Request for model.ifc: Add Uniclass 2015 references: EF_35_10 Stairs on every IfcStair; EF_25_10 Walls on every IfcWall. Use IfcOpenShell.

First a look at what the model holds.

```python
import ifcopenshell

model = ifcopenshell.open("model.ifc")
print(model.schema)
print("classifications:", [c.Name for c in model.by_type("IfcClassification")])
for ifc_class in ("IfcDoor", "IfcRoof", "IfcStair", "IfcWall", "IfcWindow"):
    print(ifc_class, len(model.by_type(ifc_class)))
```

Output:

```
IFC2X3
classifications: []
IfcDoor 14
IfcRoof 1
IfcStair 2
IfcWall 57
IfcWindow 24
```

```python
import ifcopenshell
import ifcopenshell.api.classification

model = ifcopenshell.open("model.ifc")

# IFC2X3 requires Source and Edition and has no link from the project to the system.
system = model.create_entity("IfcClassification", Source="NBS", Edition="2015", Name="Uniclass 2015")

codes = {
    "IfcStair": ("EF_35_10", "Stairs"),
    "IfcWall": ("EF_25_10", "Walls"),
}
for ifc_class, (code, name) in codes.items():
    products = model.by_type(ifc_class)
    ifcopenshell.api.classification.add_reference(
        model, products=products, classification=system, identification=code, name=name
    )
    print(code, len(products))

model.write("model-out.ifc")
```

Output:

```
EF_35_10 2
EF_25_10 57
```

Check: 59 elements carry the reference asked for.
